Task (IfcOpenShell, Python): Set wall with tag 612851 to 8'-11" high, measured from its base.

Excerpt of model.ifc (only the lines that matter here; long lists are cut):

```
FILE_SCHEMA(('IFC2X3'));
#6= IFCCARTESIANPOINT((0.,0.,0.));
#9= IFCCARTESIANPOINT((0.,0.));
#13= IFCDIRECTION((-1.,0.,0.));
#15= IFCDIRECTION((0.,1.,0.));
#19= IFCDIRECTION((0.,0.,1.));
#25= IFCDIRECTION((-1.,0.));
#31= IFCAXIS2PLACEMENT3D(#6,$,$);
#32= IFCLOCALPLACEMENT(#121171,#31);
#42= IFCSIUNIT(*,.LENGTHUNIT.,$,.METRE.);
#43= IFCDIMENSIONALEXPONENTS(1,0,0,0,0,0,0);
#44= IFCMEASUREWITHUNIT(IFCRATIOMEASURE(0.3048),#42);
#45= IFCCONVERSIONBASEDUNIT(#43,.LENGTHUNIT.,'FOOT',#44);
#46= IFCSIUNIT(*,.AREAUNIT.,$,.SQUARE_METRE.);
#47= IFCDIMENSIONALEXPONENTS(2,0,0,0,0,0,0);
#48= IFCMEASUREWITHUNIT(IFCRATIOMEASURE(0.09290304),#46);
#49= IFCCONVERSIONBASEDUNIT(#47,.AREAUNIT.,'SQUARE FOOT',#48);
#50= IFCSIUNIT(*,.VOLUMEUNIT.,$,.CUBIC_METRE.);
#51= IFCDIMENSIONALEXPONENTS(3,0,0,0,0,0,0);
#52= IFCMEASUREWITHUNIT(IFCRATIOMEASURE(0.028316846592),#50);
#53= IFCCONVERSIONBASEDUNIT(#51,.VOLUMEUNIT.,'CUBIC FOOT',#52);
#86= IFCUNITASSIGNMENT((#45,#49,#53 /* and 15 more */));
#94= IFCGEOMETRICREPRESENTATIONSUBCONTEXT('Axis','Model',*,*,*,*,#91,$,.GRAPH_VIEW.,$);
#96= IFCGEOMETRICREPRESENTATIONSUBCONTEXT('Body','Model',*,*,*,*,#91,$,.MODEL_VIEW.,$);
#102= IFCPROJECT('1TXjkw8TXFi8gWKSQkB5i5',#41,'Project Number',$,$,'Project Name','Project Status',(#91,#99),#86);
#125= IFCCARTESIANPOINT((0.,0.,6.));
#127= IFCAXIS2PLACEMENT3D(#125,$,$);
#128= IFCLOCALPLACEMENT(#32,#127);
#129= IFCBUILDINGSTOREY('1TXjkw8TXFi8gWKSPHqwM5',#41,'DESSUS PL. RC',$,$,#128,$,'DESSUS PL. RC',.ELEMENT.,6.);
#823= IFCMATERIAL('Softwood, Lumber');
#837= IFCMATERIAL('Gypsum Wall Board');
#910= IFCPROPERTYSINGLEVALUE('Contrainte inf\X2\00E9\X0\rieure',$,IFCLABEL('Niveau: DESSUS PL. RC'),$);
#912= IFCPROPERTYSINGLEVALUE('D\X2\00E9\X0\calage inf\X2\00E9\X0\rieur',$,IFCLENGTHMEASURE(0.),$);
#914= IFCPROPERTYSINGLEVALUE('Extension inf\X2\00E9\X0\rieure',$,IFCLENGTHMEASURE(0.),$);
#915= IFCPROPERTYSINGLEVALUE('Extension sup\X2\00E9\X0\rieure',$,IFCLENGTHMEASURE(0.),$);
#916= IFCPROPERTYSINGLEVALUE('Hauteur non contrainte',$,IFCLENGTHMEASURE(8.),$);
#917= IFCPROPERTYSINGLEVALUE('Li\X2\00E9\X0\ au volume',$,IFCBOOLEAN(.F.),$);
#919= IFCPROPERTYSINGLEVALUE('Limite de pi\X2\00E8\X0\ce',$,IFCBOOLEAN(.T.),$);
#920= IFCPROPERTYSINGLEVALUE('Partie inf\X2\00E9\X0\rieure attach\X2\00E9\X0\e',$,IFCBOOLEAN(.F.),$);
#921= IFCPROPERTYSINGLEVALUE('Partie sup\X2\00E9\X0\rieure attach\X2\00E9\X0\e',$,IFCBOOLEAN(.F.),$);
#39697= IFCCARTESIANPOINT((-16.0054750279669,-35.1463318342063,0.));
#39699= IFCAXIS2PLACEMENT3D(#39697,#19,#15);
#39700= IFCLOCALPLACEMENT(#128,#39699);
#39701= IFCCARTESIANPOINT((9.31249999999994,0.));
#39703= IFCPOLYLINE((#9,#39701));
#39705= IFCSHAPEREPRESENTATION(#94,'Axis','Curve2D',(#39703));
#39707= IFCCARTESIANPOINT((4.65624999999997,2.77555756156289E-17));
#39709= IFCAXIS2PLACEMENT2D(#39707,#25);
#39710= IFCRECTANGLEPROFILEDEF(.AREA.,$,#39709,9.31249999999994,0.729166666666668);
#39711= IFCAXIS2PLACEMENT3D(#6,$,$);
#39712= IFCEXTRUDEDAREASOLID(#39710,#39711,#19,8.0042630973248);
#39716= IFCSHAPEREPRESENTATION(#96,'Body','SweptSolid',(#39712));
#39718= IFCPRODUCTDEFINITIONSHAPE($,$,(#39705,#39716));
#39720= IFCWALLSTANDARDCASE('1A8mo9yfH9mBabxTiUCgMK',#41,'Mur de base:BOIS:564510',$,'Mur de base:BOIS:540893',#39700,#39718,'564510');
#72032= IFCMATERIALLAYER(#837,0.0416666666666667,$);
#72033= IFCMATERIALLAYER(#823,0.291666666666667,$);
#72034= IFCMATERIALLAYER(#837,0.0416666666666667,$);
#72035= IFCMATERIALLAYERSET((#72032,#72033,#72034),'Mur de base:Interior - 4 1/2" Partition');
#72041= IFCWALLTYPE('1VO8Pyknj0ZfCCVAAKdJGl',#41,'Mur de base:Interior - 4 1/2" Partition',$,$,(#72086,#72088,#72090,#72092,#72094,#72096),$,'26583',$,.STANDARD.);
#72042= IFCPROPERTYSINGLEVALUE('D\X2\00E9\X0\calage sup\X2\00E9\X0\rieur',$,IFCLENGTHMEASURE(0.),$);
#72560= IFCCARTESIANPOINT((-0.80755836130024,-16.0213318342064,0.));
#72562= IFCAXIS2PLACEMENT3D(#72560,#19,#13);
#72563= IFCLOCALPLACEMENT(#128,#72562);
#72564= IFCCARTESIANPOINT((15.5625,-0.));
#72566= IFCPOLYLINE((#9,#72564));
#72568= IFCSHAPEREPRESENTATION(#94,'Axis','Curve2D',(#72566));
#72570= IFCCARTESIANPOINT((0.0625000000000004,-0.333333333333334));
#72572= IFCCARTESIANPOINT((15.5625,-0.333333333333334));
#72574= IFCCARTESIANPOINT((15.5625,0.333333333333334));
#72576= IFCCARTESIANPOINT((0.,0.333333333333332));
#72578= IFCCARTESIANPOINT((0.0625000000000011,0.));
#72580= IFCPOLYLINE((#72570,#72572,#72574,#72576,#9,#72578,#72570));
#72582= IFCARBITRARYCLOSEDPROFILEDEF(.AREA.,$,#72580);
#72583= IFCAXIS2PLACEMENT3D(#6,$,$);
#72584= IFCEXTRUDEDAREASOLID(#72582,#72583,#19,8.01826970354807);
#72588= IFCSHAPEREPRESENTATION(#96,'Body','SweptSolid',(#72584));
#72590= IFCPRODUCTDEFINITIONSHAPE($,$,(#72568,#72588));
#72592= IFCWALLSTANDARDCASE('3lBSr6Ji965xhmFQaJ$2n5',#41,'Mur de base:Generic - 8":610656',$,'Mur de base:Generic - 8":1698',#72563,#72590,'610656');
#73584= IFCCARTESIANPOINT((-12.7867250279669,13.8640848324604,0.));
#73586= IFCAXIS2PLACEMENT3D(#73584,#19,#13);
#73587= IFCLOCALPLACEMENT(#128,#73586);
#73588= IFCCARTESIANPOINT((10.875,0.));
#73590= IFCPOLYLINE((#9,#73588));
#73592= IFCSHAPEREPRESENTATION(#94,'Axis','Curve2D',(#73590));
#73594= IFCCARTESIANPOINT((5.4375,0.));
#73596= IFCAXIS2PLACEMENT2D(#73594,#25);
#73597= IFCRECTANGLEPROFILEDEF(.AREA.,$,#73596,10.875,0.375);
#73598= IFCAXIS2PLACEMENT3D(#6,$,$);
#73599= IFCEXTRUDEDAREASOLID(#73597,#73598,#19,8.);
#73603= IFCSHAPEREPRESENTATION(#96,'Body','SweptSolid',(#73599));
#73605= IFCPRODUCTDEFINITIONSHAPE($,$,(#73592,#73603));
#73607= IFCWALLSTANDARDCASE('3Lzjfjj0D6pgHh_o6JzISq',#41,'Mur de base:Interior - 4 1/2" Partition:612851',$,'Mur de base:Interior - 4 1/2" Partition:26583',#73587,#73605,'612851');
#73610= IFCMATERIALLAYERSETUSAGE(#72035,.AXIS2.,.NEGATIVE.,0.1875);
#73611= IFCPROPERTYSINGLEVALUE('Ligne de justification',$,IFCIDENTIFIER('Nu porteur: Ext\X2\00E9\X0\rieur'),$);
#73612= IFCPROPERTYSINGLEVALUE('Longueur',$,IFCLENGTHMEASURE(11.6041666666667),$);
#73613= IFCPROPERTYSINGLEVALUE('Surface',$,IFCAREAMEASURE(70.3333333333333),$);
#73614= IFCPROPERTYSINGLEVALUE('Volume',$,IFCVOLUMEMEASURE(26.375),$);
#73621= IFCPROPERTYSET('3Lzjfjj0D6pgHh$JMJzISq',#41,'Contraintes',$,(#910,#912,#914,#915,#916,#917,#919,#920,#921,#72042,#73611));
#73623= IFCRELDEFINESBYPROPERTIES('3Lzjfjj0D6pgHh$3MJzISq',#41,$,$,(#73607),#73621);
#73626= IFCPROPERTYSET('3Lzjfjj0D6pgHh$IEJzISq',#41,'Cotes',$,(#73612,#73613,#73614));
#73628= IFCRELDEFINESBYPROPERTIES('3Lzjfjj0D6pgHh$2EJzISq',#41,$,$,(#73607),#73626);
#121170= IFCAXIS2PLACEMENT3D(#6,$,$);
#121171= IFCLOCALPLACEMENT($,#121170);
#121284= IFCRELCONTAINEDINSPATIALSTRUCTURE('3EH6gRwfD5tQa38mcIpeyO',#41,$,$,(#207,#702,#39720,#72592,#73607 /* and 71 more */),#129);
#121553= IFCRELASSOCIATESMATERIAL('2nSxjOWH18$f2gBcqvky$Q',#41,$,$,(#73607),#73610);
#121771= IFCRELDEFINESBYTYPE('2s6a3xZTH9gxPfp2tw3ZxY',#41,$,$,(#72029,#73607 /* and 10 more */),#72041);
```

```python
import ifcopenshell
import ifcopenshell.api.pset
import ifcopenshell.geom
import ifcopenshell.util.element
import ifcopenshell.util.representation
import ifcopenshell.util.shape
import ifcopenshell.util.unit

model = ifcopenshell.open("model.ifc")
unit_scale = ifcopenshell.util.unit.calculate_unit_scale(model)
area_scale = ifcopenshell.util.unit.calculate_unit_scale(model, "AREAUNIT")
volume_scale = ifcopenshell.util.unit.calculate_unit_scale(model, "VOLUMEUNIT")
settings = ifcopenshell.geom.settings()


def volume(element):
    """Net volume in cubic metres, openings subtracted."""
    shape = ifcopenshell.geom.create_shape(settings, element)
    return ifcopenshell.util.shape.get_volume(shape.geometry)


wall = model.by_id(73607)
before = volume(wall)

body = ifcopenshell.util.representation.get_representation(wall, "Model", "Body")
solid = body.Items[0]
old_height = solid.Depth
solid.Depth = 107 * 0.0254 / unit_scale
after = volume(wall)
thickness = 0.1143  # wall thickness in metres

# Update the stored height, areas and volumes.
pset = model.by_id(ifcopenshell.util.element.get_pset(wall, "Contraintes", should_inherit=False)["id"])
ifcopenshell.api.pset.edit_pset(model, pset=pset, properties={
    "Hauteur non contrainte": model.create_entity("IfcLengthMeasure", solid.Depth),
})
pset = model.by_id(ifcopenshell.util.element.get_pset(wall, "Cotes", should_inherit=False)["id"])
ifcopenshell.api.pset.edit_pset(model, pset=pset, properties={
    "Surface": model.create_entity("IfcAreaMeasure", after / thickness / area_scale),
    "Volume": model.create_entity("IfcVolumeMeasure", after / volume_scale),
})

print(f"height {old_height:g} -> {solid.Depth:g}, volume {before:.3f} -> {after:.3f} m3")

model.write("model_edited.ifc")
```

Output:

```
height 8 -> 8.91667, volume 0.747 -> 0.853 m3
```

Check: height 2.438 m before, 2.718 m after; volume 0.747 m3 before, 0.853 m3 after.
